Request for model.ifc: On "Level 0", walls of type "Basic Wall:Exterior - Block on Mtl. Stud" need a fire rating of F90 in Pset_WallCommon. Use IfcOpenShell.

First a look at what the model holds.

```python
import ifcopenshell
import ifcopenshell.util.element

model = ifcopenshell.open("model.ifc")
print(model.schema)
storey = next(s for s in model.by_type("IfcBuildingStorey") if s.Name == "Level 0")
walls = [e for e in ifcopenshell.util.element.get_decomposition(storey) if e.is_a("IfcWall")]
seen = {}
for e in walls:
    element_type = ifcopenshell.util.element.get_type(e)
    key = (element_type.Name if element_type != e and element_type else None, ifcopenshell.util.element.get_pset(e, "Pset_WallCommon", "FireRating"))
    seen[key] = seen.get(key, 0) + 1
for (name, value), count in sorted(seen.items(), key=str):
    print(count, "x", name, "|", value)
```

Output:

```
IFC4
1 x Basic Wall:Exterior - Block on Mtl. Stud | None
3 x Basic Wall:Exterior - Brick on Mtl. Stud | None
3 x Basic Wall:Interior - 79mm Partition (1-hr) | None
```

```python
import ifcopenshell
import ifcopenshell.api.pset
import ifcopenshell.util.element

model = ifcopenshell.open("model.ifc")

storey = next(s for s in model.by_type("IfcBuildingStorey") if s.Name == "Level 0")
walls = [e for e in ifcopenshell.util.element.get_decomposition(storey) if e.is_a("IfcWall")]

count = 0
for e in walls:
    element_type = ifcopenshell.util.element.get_type(e)
    if element_type in (None, e) or element_type.Name != "Basic Wall:Exterior - Block on Mtl. Stud":
        continue
    # add_pset returns the element's existing set when there is one.
    pset = ifcopenshell.api.pset.add_pset(model, product=e, name="Pset_WallCommon")
    ifcopenshell.api.pset.edit_pset(model, pset=pset, properties={"FireRating": "F90"})
    count += 1

print(count, "walls updated")

model.write("model_v2.ifc")
```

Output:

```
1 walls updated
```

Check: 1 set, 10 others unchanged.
